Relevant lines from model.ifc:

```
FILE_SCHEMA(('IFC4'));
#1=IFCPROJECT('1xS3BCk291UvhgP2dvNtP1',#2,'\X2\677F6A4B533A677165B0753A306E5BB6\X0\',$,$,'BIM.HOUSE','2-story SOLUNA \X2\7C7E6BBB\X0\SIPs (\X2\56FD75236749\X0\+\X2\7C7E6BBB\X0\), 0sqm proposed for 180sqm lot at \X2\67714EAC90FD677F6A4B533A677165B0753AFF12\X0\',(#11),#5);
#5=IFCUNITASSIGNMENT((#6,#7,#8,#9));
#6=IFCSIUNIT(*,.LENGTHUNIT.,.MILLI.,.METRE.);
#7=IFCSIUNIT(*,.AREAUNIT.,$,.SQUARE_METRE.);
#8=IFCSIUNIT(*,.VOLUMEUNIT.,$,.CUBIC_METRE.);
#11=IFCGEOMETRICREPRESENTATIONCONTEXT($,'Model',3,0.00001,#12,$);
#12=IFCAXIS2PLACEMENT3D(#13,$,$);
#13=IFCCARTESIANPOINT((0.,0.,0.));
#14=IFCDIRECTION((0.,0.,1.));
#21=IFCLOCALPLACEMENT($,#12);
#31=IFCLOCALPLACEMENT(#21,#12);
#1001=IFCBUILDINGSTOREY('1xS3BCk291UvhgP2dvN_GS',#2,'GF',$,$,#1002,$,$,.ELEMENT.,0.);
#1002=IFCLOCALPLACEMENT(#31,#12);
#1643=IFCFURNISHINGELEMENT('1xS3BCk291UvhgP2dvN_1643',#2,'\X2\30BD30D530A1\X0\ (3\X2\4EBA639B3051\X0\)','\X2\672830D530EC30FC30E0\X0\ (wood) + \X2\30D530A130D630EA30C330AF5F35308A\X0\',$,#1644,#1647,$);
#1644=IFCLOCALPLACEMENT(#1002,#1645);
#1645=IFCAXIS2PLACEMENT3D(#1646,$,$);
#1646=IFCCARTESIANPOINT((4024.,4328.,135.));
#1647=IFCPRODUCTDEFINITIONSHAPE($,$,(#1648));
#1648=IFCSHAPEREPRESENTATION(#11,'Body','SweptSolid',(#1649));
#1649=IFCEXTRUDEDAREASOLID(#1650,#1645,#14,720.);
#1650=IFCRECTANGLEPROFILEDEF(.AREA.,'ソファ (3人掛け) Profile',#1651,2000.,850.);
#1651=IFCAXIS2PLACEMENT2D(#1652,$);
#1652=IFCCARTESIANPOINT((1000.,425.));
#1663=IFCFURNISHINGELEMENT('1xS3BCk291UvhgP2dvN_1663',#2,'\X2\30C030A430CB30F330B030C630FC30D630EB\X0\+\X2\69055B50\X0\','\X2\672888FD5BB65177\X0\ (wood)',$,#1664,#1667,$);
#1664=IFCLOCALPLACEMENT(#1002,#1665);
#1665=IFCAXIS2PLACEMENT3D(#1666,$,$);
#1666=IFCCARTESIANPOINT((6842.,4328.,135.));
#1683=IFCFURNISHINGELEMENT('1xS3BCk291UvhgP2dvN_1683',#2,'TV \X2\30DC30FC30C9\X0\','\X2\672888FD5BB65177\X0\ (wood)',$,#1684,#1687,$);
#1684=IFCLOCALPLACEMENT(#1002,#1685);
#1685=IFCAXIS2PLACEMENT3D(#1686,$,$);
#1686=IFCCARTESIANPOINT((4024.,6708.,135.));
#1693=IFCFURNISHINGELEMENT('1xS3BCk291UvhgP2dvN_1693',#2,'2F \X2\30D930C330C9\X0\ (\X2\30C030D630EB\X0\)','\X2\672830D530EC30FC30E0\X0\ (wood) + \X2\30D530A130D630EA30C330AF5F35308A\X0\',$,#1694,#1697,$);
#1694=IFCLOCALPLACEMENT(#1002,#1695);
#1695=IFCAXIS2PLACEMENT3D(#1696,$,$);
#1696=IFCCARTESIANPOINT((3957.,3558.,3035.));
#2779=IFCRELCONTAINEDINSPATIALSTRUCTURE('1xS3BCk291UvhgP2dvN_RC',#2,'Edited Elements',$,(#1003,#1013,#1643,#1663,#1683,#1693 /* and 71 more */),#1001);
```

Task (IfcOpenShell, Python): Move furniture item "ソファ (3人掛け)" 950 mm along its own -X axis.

```python
import ifcopenshell
import ifcopenshell.api.geometry
import ifcopenshell.util.placement
import ifcopenshell.util.unit

model = ifcopenshell.open("model.ifc")
unit_scale = ifcopenshell.util.unit.calculate_unit_scale(model)

item = model.by_guid("1xS3BCk291UvhgP2dvN_1643")
matrix = ifcopenshell.util.placement.get_local_placement(item.ObjectPlacement)
matrix[:3, 3] -= matrix[:3, 0] * 0.95 / unit_scale
ifcopenshell.api.geometry.edit_object_placement(model, product=item, matrix=matrix, is_si=False)

print(ifcopenshell.util.placement.get_local_placement(item.ObjectPlacement).round(3) + 0.0)

model.write("model_rev.ifc")
```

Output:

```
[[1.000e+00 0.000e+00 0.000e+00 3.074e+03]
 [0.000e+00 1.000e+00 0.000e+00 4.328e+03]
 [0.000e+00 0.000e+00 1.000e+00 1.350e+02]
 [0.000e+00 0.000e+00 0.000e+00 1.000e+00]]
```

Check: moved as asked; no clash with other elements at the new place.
